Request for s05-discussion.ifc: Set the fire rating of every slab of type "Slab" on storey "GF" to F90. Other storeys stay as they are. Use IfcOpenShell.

First a look at what the model holds.

```python
import ifcopenshell
import ifcopenshell.util.element

model = ifcopenshell.open("s05-discussion.ifc")
print(model.schema)
storey = next(s for s in model.by_type("IfcBuildingStorey") if s.Name == "GF")
slabs = [e for e in ifcopenshell.util.element.get_decomposition(storey) if e.is_a("IfcSlab")]
seen = {}
for e in slabs:
    element_type = ifcopenshell.util.element.get_type(e)
    key = (element_type.Name if element_type != e and element_type else None, ifcopenshell.util.element.get_pset(e, "Pset_SlabCommon", "FireRating"))
    seen[key] = seen.get(key, 0) + 1
for (name, value), count in sorted(seen.items(), key=str):
    print(count, "x", name, "|", value)
```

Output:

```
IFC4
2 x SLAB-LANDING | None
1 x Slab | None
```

```python
import ifcopenshell
import ifcopenshell.api.pset
import ifcopenshell.util.element

model = ifcopenshell.open("s05-discussion.ifc")

storey = next(s for s in model.by_type("IfcBuildingStorey") if s.Name == "GF")
slabs = [e for e in ifcopenshell.util.element.get_decomposition(storey) if e.is_a("IfcSlab")]

count = 0
for e in slabs:
    element_type = ifcopenshell.util.element.get_type(e)
    if element_type in (None, e) or element_type.Name != "Slab":
        continue
    # add_pset returns the element's existing set when there is one.
    pset = ifcopenshell.api.pset.add_pset(model, product=e, name="Pset_SlabCommon")
    ifcopenshell.api.pset.edit_pset(model, pset=pset, properties={"FireRating": "F90"})
    count += 1

print(count, "slabs updated")

model.write("s05-discussion_v2.ifc")
```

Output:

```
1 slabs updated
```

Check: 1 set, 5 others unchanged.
